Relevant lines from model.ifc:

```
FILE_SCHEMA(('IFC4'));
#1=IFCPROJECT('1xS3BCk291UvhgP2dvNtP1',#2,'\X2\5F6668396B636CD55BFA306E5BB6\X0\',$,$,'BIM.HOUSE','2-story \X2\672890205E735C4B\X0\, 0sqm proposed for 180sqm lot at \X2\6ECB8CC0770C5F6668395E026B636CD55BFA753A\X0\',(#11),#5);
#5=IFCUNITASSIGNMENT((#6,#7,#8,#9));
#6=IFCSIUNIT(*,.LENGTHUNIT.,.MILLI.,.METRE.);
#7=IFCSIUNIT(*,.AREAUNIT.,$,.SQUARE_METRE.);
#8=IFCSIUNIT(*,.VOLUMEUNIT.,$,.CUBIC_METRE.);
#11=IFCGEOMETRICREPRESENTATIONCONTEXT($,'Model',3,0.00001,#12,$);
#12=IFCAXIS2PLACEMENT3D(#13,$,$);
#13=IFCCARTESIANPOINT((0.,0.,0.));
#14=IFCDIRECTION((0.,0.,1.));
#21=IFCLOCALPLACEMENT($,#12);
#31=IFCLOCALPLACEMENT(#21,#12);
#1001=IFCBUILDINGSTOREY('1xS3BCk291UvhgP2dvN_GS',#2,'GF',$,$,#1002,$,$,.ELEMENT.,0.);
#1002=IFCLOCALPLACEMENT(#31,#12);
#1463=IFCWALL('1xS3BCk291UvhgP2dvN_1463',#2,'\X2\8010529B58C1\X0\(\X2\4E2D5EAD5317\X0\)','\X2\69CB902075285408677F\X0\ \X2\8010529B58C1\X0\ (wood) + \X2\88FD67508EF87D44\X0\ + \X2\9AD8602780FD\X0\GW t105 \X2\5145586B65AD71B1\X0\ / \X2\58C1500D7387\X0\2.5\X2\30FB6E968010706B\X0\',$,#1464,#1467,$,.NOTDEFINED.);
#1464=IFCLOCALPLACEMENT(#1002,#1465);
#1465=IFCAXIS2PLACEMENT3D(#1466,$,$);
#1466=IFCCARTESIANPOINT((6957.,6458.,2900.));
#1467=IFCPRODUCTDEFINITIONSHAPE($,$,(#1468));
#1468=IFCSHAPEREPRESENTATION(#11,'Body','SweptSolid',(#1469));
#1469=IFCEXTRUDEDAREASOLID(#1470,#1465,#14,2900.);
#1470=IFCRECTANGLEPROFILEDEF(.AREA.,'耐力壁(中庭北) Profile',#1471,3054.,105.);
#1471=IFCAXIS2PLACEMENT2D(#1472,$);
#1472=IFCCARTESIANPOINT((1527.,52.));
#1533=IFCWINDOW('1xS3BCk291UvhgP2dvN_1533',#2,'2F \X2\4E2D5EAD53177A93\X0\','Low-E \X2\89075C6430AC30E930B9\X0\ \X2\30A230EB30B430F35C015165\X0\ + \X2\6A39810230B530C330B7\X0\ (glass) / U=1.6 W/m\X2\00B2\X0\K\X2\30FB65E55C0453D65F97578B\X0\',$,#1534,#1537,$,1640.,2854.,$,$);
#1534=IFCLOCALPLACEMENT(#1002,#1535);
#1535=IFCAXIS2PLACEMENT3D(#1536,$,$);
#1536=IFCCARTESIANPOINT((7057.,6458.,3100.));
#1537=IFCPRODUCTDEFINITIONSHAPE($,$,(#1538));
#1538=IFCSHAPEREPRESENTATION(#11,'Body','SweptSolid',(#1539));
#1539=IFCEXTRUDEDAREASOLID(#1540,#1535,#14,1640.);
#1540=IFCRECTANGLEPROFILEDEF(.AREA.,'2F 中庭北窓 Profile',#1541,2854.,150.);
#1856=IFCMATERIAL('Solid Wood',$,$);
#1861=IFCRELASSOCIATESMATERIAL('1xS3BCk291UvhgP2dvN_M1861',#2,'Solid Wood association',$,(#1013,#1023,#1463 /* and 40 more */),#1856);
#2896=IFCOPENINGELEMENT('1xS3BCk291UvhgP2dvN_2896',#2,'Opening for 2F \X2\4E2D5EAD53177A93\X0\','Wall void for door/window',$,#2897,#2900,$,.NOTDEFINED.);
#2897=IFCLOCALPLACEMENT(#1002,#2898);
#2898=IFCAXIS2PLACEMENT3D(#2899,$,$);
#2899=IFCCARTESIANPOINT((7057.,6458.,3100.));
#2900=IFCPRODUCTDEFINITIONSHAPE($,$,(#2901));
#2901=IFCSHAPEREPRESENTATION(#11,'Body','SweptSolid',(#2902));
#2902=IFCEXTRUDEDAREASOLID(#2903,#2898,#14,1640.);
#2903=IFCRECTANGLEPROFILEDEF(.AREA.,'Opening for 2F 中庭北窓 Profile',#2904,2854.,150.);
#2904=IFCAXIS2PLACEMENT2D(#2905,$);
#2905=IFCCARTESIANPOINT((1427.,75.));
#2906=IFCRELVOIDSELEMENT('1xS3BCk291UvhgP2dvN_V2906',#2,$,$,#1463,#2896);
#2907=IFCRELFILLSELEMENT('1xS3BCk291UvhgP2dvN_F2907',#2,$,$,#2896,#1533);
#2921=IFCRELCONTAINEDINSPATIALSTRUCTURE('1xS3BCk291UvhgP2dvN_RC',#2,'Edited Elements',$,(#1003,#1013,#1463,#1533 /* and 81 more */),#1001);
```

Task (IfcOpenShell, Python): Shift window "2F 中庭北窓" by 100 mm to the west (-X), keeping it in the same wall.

```python
import ifcopenshell
import ifcopenshell.api.geometry
import ifcopenshell.util.placement

model = ifcopenshell.open("model.ifc")

window = model.by_guid("1xS3BCk291UvhgP2dvN_1533")
opening = window.FillsVoids[0].RelatingOpeningElement
wall = opening.VoidsElements[0].RelatingBuildingElement

wall_matrix = ifcopenshell.util.placement.get_local_placement(wall.ObjectPlacement)
shift = wall_matrix[:3, 0] * -100.0
before = ifcopenshell.util.placement.get_local_placement(window.ObjectPlacement)[:3, 3].copy()

# The window is not placed relative to its opening, so move both.
for product in (opening, window):
    matrix = ifcopenshell.util.placement.get_local_placement(product.ObjectPlacement)
    matrix[:3, 3] += shift
    ifcopenshell.api.geometry.edit_object_placement(model, product=product, matrix=matrix, is_si=False)

after = ifcopenshell.util.placement.get_local_placement(window.ObjectPlacement)[:3, 3]
print("window moved by", (after - before).round(3) + 0.0)

model.write("model_updated.ifc")
```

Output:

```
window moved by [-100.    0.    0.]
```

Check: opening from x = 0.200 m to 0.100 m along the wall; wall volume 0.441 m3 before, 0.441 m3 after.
